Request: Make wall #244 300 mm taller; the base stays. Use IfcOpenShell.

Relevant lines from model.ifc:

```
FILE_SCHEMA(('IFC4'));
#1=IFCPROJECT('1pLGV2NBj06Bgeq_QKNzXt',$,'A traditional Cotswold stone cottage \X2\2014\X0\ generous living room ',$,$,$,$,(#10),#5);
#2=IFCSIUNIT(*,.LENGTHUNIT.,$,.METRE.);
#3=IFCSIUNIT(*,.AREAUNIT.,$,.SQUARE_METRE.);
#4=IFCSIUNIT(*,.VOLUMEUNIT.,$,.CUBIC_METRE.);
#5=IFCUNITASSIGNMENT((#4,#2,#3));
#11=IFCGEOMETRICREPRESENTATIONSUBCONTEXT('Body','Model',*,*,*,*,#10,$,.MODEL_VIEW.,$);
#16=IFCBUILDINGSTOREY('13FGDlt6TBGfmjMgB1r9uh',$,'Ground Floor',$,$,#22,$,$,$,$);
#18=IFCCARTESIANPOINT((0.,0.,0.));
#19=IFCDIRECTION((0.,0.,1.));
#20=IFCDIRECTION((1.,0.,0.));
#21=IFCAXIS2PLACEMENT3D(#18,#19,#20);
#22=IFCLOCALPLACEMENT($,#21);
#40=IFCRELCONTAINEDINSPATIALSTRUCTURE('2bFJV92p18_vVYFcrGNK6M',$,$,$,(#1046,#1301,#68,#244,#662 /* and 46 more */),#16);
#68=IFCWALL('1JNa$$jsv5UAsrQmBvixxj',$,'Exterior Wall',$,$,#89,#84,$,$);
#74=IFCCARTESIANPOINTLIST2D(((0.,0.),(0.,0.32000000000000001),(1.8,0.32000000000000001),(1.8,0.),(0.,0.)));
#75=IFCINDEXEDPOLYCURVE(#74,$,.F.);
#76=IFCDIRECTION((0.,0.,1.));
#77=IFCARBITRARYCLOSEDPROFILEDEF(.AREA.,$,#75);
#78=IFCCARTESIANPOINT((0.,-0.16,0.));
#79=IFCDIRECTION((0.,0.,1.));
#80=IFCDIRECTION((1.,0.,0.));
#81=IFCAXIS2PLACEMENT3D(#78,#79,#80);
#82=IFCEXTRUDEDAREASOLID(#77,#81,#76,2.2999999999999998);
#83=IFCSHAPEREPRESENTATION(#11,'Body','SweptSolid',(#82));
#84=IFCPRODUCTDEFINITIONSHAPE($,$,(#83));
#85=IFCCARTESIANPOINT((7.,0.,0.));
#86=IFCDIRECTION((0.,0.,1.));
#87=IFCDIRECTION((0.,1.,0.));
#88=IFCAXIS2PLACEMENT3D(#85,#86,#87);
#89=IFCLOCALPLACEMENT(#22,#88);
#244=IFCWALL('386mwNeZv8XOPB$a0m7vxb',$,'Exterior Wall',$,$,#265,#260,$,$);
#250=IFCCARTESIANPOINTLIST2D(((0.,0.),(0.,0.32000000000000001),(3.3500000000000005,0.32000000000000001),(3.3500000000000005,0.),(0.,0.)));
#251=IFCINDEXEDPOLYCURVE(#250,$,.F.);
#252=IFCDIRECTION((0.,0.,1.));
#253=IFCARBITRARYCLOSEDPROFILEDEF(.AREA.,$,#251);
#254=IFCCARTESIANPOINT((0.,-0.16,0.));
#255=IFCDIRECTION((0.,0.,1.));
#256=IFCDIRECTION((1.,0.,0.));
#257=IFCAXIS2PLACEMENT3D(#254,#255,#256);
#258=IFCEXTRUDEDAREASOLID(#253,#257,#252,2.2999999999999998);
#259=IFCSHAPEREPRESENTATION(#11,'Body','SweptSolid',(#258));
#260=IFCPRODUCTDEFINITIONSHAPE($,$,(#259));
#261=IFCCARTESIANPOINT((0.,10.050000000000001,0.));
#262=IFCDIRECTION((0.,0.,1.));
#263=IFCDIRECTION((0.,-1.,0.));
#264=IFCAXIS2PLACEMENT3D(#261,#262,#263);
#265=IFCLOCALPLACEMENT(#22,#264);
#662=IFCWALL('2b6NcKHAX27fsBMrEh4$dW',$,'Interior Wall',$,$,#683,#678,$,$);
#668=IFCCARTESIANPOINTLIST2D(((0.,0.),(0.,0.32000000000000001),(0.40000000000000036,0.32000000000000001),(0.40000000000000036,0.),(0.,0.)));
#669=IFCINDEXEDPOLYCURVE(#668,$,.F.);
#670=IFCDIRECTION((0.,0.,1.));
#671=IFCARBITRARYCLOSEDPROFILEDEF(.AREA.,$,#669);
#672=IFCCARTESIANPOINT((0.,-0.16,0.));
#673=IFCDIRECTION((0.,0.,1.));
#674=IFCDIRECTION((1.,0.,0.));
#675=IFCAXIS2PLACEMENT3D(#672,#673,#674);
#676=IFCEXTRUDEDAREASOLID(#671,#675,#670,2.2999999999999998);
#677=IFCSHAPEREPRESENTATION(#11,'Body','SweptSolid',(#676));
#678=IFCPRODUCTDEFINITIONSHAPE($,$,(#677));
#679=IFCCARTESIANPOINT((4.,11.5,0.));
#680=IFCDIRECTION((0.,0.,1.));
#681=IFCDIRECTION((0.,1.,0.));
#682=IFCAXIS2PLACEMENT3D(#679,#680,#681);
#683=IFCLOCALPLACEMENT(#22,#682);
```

```python
import ifcopenshell
import ifcopenshell.geom
import ifcopenshell.util.representation
import ifcopenshell.util.shape
import ifcopenshell.util.unit

model = ifcopenshell.open("model.ifc")
unit_scale = ifcopenshell.util.unit.calculate_unit_scale(model)
settings = ifcopenshell.geom.settings()


def volume(element):
    """Net volume in cubic metres, openings subtracted."""
    shape = ifcopenshell.geom.create_shape(settings, element)
    return ifcopenshell.util.shape.get_volume(shape.geometry)


wall = model.by_guid("386mwNeZv8XOPB$a0m7vxb")
before = volume(wall)

body = ifcopenshell.util.representation.get_representation(wall, "Model", "Body")
solid = body.Items[0]
old_height = solid.Depth
solid.Depth += 0.3 / unit_scale
after = volume(wall)

print(f"height {old_height:g} -> {solid.Depth:g}, volume {before:.3f} -> {after:.3f} m3")

model.write("model_rev.ifc")
```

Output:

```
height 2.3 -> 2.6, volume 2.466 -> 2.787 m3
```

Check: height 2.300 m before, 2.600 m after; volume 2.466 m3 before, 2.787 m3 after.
